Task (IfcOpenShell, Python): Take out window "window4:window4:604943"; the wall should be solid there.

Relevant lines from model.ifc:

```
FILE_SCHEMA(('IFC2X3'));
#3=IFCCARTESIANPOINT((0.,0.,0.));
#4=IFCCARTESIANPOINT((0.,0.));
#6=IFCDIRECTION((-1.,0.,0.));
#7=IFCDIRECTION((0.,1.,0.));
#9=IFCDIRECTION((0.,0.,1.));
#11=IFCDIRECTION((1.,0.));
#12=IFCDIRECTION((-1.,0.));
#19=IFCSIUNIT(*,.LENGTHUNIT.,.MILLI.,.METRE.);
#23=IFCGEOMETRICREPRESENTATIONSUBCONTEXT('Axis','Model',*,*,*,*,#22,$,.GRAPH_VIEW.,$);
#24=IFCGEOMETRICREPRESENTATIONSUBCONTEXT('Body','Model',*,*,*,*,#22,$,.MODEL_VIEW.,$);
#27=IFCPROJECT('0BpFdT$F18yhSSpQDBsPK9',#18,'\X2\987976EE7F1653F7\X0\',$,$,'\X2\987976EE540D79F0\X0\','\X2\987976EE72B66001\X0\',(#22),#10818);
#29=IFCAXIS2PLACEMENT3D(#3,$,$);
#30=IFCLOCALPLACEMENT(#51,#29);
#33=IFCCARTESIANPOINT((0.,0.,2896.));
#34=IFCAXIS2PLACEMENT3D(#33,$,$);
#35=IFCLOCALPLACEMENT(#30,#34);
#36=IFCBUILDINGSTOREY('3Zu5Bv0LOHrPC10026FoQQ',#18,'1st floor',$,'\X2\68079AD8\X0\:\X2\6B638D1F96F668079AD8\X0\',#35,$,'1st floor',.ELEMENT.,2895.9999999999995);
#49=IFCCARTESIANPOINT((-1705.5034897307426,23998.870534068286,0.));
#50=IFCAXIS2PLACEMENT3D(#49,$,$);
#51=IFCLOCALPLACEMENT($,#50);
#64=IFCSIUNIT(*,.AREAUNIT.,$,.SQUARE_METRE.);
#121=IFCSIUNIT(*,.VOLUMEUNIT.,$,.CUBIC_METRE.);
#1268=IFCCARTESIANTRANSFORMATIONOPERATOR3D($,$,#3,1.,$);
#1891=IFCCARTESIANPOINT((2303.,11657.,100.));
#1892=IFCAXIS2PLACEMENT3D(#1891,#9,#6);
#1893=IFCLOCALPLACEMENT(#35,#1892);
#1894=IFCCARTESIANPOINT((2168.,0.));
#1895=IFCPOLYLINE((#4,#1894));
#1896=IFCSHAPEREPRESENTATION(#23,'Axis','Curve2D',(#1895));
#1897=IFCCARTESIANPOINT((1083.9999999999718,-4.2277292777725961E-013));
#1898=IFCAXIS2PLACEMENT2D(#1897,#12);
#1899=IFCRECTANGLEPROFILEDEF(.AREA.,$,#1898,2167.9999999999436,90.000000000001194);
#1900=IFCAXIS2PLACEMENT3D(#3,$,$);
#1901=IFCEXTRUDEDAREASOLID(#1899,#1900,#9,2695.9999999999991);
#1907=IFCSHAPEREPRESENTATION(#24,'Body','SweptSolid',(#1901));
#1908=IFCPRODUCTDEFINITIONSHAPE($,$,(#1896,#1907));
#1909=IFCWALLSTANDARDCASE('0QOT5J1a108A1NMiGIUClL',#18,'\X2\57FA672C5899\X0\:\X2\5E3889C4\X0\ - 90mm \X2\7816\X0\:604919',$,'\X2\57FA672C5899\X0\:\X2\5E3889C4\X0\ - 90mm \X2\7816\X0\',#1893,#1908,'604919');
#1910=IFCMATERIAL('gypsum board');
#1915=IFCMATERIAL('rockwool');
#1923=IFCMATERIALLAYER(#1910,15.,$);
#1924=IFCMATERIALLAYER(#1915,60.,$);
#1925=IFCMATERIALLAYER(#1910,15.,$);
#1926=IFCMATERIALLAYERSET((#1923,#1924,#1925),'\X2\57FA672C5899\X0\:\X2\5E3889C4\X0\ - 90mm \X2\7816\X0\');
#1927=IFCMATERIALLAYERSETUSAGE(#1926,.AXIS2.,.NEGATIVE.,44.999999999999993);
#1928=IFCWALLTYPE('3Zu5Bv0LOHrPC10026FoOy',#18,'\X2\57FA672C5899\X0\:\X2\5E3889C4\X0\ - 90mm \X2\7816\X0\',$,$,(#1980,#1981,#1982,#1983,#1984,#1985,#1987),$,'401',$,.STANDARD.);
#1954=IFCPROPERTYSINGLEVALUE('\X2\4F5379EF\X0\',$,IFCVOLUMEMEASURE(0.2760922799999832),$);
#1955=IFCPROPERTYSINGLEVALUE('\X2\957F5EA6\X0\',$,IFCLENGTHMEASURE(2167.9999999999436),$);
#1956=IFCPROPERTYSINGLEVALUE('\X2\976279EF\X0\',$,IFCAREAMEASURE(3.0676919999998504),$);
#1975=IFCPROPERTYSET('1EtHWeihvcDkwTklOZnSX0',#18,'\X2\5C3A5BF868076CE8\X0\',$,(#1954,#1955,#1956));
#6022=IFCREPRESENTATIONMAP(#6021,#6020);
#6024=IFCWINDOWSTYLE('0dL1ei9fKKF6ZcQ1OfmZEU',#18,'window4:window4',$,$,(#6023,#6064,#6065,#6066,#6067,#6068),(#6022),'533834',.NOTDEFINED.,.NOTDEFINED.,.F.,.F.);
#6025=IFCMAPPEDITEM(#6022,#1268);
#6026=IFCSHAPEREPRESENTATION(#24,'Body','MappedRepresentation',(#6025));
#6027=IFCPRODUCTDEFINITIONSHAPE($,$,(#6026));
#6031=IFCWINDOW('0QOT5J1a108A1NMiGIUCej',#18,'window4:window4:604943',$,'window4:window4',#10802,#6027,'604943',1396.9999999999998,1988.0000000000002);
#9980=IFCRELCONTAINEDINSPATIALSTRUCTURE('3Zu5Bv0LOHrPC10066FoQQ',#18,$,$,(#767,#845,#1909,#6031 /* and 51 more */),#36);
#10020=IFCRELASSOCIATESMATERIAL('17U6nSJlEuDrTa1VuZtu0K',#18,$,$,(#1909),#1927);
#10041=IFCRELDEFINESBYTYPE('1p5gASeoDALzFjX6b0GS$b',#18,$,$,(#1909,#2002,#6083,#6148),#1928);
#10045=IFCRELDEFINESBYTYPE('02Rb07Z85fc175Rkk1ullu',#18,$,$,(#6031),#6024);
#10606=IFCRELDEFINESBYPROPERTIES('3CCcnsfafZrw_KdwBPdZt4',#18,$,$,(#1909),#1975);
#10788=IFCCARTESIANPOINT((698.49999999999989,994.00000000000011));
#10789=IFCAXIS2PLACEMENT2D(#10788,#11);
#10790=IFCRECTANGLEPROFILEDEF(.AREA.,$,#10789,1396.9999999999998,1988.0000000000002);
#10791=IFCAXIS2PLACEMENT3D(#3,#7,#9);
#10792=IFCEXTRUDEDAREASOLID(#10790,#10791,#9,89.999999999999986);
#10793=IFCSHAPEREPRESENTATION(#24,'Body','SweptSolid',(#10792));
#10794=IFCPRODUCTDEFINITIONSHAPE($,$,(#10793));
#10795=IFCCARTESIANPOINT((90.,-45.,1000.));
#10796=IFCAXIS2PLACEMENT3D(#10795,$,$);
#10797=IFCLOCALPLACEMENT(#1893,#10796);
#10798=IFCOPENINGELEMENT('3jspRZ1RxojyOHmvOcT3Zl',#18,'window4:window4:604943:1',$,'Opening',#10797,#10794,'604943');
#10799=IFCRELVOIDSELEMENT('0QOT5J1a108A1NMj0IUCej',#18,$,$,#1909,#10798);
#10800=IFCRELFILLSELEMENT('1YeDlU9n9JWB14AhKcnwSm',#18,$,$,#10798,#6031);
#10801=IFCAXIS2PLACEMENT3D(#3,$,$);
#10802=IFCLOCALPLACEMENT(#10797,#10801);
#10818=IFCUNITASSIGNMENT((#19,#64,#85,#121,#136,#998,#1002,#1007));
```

```python
import ifcopenshell
import ifcopenshell.api.feature
import ifcopenshell.api.pset
import ifcopenshell.api.root
import ifcopenshell.geom
import ifcopenshell.util.element
import ifcopenshell.util.shape
import ifcopenshell.util.unit

model = ifcopenshell.open("model.ifc")
area_scale = ifcopenshell.util.unit.calculate_unit_scale(model, "AREAUNIT")
volume_scale = ifcopenshell.util.unit.calculate_unit_scale(model, "VOLUMEUNIT")
settings = ifcopenshell.geom.settings()


def volume(element):
    """Net volume in cubic metres, openings subtracted."""
    shape = ifcopenshell.geom.create_shape(settings, element)
    return ifcopenshell.util.shape.get_volume(shape.geometry)


window = model.by_guid("0QOT5J1a108A1NMiGIUCej")
opening = window.FillsVoids[0].RelatingOpeningElement
wall = opening.VoidsElements[0].RelatingBuildingElement
before = volume(wall)

ifcopenshell.api.root.remove_product(model, product=window)
ifcopenshell.api.feature.remove_feature(model, feature=opening)

after = volume(wall)
thickness = 0.09  # wall thickness in metres

# Update the wall's stored quantities.
pset = model.by_id(ifcopenshell.util.element.get_pset(wall, "尺寸标注", should_inherit=False)["id"])
ifcopenshell.api.pset.edit_pset(model, pset=pset, properties={
    "体积": model.create_entity("IfcVolumeMeasure", after / volume_scale),
    "面积": model.create_entity("IfcAreaMeasure", after / thickness / area_scale),
})

print(f"wall volume {before:.3f} -> {after:.3f} m3")

model.write("model_updated.ifc")
```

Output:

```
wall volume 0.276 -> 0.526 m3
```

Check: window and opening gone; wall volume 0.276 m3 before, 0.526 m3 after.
